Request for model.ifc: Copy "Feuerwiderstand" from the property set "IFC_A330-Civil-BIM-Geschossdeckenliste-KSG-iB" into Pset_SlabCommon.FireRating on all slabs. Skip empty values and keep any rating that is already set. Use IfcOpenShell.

First a look at what the model holds.

```python
import ifcopenshell
import ifcopenshell.util.element

model = ifcopenshell.open("model.ifc")
print(model.schema)
slabs = model.by_type("IfcSlab")
print(len(slabs), "slabs")
for e in slabs[:8]:
    source = ifcopenshell.util.element.get_pset(e, "IFC_A330-Civil-BIM-Geschossdeckenliste-KSG-iB", "Feuerwiderstand")
    target = ifcopenshell.util.element.get_pset(e, "Pset_SlabCommon", "FireRating")
    print(e.id(), repr(source), repr(target), sep=" | ")
```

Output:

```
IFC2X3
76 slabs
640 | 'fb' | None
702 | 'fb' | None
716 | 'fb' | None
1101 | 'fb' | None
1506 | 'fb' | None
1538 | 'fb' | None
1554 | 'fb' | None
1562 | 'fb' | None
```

```python
import ifcopenshell
import ifcopenshell.api.pset
import ifcopenshell.util.element

model = ifcopenshell.open("model.ifc")

count = 0
for e in model.by_type("IfcSlab"):
    value = ifcopenshell.util.element.get_pset(e, "IFC_A330-Civil-BIM-Geschossdeckenliste-KSG-iB", "Feuerwiderstand")
    current = ifcopenshell.util.element.get_pset(e, "Pset_SlabCommon", "FireRating")
    if not value or not value.strip() or current:
        continue
    found = ifcopenshell.util.element.get_pset(e, "Pset_SlabCommon", should_inherit=False)
    if found:
        pset = model.by_id(found["id"])
        if len(ifcopenshell.util.element.get_elements_by_pset(pset)) > 1:
            pset = ifcopenshell.api.pset.unshare_pset(model, products=[e], pset=pset)[0]
    else:
        pset = ifcopenshell.api.pset.add_pset(model, product=e, name="Pset_SlabCommon")
    ifcopenshell.api.pset.edit_pset(model, pset=pset, properties={"FireRating": value})
    count += 1

print(count, "slabs updated")

model.write("model_rev.ifc")
```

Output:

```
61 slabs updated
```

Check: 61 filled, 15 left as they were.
